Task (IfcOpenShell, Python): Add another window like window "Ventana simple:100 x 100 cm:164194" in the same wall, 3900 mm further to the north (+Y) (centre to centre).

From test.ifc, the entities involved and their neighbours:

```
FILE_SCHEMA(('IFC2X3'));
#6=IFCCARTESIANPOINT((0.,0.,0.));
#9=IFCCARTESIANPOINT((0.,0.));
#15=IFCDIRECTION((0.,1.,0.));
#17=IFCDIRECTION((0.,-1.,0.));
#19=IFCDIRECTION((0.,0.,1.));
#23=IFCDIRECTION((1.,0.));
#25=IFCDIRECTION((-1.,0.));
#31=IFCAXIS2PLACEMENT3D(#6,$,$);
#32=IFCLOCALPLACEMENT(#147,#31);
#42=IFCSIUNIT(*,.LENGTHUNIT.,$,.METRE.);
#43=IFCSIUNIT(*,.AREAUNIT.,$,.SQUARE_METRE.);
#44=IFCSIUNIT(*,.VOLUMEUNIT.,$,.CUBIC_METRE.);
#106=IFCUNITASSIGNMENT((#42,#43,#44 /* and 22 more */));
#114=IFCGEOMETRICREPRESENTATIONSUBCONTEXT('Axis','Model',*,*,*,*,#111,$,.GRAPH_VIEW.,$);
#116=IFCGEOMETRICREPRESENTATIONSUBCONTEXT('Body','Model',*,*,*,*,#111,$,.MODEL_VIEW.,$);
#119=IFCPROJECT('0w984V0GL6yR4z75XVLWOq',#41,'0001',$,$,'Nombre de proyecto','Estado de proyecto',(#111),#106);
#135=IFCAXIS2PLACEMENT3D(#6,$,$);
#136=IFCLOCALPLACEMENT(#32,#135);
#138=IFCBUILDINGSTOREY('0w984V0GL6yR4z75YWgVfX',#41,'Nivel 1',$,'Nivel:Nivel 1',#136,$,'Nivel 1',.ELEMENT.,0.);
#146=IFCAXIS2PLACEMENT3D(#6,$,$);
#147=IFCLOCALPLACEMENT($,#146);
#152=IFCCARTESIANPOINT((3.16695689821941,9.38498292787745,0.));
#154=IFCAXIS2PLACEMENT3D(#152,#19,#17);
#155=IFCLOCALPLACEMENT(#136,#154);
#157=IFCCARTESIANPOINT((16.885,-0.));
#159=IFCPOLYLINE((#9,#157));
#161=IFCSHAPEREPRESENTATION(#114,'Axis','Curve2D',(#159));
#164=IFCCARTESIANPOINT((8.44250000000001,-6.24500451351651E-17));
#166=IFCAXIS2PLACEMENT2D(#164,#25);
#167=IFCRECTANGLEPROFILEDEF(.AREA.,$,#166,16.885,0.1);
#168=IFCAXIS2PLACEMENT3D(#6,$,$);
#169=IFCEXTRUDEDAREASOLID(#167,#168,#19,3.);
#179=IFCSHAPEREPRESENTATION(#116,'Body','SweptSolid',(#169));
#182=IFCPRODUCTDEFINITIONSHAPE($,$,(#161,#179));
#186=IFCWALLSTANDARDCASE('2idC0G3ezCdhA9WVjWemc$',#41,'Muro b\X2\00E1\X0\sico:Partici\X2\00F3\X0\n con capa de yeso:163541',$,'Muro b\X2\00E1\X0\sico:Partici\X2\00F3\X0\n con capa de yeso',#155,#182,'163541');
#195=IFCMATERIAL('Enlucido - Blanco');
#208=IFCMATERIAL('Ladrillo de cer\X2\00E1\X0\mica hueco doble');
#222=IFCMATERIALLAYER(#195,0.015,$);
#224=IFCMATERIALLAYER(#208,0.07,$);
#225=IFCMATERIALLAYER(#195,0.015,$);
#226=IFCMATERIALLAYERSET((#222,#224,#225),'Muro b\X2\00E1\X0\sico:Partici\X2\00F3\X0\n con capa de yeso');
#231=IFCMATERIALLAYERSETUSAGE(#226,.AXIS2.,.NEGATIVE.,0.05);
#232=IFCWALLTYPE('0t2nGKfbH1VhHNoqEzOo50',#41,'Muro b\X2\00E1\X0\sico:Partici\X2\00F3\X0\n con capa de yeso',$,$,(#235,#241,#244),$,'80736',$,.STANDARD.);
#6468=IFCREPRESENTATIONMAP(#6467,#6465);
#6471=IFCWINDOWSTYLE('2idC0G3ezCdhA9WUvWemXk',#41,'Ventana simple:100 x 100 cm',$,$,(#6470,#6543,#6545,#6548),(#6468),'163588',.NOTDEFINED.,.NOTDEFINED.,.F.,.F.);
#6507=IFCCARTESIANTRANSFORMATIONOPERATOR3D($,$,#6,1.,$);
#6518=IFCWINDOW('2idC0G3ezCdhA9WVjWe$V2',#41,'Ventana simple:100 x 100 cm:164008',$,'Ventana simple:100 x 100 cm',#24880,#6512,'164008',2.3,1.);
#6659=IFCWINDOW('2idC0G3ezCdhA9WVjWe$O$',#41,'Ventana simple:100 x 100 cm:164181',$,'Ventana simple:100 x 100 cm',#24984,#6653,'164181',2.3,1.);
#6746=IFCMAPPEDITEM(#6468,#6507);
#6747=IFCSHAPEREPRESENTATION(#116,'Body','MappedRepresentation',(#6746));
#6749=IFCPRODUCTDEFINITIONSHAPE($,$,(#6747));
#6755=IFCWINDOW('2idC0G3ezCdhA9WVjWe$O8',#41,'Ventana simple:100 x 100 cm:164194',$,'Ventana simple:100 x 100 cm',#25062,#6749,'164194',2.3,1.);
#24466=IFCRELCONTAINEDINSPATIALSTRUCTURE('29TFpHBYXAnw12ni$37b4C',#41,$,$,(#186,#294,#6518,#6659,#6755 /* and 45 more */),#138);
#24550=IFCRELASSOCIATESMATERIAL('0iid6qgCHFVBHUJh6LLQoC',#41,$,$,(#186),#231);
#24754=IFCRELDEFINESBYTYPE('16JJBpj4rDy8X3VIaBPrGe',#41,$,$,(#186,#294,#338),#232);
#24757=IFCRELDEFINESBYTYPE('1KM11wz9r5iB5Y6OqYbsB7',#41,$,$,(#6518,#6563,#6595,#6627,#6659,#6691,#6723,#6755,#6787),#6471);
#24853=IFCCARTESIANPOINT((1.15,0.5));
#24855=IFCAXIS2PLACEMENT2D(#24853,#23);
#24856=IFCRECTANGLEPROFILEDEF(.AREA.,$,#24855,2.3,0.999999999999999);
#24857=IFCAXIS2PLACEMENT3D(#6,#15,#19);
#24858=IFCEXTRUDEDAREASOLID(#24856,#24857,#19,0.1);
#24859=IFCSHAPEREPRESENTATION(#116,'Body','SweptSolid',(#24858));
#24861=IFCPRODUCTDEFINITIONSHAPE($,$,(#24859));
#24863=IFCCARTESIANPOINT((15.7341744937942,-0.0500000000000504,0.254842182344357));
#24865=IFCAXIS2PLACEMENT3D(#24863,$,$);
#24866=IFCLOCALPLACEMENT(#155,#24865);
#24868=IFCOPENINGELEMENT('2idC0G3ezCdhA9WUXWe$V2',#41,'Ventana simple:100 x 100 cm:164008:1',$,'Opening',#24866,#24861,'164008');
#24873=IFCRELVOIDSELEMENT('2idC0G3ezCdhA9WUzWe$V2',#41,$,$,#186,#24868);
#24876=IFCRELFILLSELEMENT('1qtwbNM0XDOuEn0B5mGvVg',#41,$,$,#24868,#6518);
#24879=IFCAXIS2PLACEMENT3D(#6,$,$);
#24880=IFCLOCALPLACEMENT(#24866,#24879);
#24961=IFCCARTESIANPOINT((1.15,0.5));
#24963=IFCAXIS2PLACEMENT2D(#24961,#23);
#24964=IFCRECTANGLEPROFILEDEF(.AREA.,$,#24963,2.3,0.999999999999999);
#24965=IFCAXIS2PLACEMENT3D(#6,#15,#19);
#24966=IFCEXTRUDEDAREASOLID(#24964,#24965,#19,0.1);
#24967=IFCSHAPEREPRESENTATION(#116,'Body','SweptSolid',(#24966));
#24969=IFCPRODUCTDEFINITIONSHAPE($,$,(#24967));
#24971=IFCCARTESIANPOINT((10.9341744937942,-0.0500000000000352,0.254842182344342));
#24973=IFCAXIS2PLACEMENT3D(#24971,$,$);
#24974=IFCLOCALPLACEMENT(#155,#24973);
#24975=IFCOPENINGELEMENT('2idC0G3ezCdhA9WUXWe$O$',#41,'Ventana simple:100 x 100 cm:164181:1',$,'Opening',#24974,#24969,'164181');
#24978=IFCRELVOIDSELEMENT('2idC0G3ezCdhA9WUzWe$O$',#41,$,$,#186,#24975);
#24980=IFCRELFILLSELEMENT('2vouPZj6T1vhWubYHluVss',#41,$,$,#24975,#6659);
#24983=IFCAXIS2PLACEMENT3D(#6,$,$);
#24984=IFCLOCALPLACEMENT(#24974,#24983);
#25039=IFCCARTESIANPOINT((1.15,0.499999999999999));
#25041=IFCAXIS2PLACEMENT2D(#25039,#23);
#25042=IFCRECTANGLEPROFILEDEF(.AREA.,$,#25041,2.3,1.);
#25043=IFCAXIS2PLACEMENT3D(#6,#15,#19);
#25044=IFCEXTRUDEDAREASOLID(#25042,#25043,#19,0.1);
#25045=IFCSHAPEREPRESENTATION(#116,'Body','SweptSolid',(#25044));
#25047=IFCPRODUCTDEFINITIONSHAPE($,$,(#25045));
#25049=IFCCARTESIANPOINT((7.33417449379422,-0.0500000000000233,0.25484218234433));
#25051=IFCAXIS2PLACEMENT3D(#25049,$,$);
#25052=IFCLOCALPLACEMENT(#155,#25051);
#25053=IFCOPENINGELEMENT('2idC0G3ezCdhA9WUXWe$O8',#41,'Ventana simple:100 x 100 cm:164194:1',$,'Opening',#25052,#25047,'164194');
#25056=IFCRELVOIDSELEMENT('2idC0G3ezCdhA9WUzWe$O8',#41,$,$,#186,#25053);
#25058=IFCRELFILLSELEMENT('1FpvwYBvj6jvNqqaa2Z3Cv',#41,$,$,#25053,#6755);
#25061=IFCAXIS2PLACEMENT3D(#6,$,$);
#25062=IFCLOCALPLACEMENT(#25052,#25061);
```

```python
import ifcopenshell
import ifcopenshell.api.feature
import ifcopenshell.api.geometry
import ifcopenshell.api.root
import ifcopenshell.geom
import ifcopenshell.util.element
import ifcopenshell.util.placement
import ifcopenshell.util.shape
import ifcopenshell.util.unit

model = ifcopenshell.open("test.ifc")
unit_scale = ifcopenshell.util.unit.calculate_unit_scale(model)
settings = ifcopenshell.geom.settings()


def volume(element):
    """Net volume in cubic metres, openings subtracted."""
    shape = ifcopenshell.geom.create_shape(settings, element)
    return ifcopenshell.util.shape.get_volume(shape.geometry)


def reuse_history(source, copy):
    """copy_class also copies each property set's owner history, people and application; keep the originals."""
    for rel in copy.IsDefinedBy:
        if rel.is_a("IfcRelDefinesByProperties") and (history := rel.RelatingPropertyDefinition.OwnerHistory):
            rel.RelatingPropertyDefinition.OwnerHistory = source.OwnerHistory
            ifcopenshell.util.element.remove_deep2(model, history)


window = model.by_guid("2idC0G3ezCdhA9WVjWe$O8")
opening = window.FillsVoids[0].RelatingOpeningElement
wall = opening.VoidsElements[0].RelatingBuildingElement
before = volume(wall)
shift = ifcopenshell.util.placement.get_local_placement(wall.ObjectPlacement)[:3, 0] * -3.9 / unit_scale

# copy_class copies the void relationship, type, container and properties, but no geometry.
new_opening = ifcopenshell.api.root.copy_class(model, product=opening)
new_opening.Representation = ifcopenshell.util.element.copy_deep(
    model, opening.Representation, exclude=["IfcGeometricRepresentationContext", "IfcRepresentationMap"]
)
new_opening.Name = "Ventana simple:100 x 100 cm"
new_opening.Tag = None
new_window = ifcopenshell.api.root.copy_class(model, product=window)
new_window.Representation = ifcopenshell.util.element.copy_deep(
    model, window.Representation, exclude=["IfcGeometricRepresentationContext", "IfcRepresentationMap"]
)
new_window.Name = "Ventana simple:100 x 100 cm"
new_window.Tag = None
reuse_history(window, new_window)
fills = ifcopenshell.api.feature.add_filling(model, opening=new_opening, element=new_window)
fills.OwnerHistory = new_window.OwnerHistory  # required in IFC2X3

for old, new in ((opening, new_opening), (window, new_window)):
    matrix = ifcopenshell.util.placement.get_local_placement(old.ObjectPlacement)
    matrix[:3, 3] += shift
    ifcopenshell.api.geometry.edit_object_placement(model, product=new, matrix=matrix, is_si=False)

after = volume(wall)

print(f"wall volume {before:.3f} -> {after:.3f} m3")

model.write("test_v2.ifc")
```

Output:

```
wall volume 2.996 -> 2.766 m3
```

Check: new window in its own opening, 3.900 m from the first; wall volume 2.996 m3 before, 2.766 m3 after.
